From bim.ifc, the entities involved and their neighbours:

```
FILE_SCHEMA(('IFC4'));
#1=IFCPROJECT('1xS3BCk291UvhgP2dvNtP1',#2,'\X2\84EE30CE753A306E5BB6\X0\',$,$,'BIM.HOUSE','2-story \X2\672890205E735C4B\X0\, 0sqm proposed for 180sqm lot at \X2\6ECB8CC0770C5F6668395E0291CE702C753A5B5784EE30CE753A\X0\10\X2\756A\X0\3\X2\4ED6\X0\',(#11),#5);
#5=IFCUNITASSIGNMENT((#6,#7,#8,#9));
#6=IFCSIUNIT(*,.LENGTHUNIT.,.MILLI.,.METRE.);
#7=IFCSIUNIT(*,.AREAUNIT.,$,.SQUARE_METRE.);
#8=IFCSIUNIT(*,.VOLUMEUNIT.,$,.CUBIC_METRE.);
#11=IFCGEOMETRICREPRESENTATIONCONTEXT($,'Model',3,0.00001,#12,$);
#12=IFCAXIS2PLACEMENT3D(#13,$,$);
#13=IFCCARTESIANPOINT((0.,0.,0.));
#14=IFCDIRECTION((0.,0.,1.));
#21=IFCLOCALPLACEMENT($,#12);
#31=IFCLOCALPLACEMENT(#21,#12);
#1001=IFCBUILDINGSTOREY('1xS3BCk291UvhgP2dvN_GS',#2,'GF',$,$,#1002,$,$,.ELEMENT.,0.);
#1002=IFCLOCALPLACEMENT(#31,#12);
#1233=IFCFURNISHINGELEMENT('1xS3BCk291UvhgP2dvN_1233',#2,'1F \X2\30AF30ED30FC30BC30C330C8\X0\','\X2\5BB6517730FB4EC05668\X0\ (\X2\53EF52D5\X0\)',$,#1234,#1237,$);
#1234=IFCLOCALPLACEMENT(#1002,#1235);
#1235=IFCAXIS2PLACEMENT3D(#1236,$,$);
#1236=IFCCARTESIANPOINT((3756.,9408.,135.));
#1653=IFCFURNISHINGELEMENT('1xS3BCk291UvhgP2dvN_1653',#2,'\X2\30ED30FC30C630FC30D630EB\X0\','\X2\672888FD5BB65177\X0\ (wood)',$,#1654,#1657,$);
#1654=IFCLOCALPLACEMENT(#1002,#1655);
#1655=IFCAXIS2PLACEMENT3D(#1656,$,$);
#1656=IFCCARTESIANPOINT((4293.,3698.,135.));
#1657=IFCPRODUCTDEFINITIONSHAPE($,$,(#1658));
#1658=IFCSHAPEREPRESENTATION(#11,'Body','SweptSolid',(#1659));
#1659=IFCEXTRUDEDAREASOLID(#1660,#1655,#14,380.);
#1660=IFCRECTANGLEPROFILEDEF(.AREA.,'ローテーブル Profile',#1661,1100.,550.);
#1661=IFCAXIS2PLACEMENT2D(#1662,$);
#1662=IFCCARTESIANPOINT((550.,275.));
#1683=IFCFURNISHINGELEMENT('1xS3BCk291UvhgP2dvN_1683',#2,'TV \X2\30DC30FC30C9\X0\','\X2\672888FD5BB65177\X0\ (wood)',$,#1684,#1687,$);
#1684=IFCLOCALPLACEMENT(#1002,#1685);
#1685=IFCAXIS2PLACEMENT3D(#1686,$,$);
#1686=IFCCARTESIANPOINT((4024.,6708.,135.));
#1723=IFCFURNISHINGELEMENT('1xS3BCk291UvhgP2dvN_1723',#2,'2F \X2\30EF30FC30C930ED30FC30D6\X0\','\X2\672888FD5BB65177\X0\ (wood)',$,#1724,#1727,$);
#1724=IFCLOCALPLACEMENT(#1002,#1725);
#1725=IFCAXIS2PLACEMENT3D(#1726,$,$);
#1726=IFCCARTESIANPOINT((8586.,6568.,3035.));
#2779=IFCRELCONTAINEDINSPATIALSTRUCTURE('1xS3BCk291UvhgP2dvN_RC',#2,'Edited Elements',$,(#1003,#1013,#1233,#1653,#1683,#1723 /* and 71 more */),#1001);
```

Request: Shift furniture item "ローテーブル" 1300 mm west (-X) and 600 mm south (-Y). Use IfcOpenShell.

```python
import ifcopenshell
import ifcopenshell.api.geometry
import ifcopenshell.util.placement

model = ifcopenshell.open("bim.ifc")

item = model.by_guid("1xS3BCk291UvhgP2dvN_1653")
matrix = ifcopenshell.util.placement.get_local_placement(item.ObjectPlacement)
matrix[0, 3] -= 1300.0
matrix[1, 3] -= 600.0
ifcopenshell.api.geometry.edit_object_placement(model, product=item, matrix=matrix, is_si=False)

print(ifcopenshell.util.placement.get_local_placement(item.ObjectPlacement).round(3) + 0.0)

model.write("bim_edited.ifc")
```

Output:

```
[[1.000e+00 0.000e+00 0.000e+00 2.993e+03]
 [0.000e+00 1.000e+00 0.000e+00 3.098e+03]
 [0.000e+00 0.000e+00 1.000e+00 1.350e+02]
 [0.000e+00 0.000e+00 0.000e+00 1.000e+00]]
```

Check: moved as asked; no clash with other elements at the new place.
